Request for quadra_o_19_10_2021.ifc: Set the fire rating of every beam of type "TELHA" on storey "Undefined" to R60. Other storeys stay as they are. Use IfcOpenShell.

First a look at what the model holds.

```python
import ifcopenshell
import ifcopenshell.util.element

model = ifcopenshell.open("quadra_o_19_10_2021.ifc")
print(model.schema)
storey = next(s for s in model.by_type("IfcBuildingStorey") if s.Name == "Undefined")
beams = [e for e in ifcopenshell.util.element.get_decomposition(storey) if e.is_a("IfcBeam")]
seen = {}
for e in beams:
    element_type = ifcopenshell.util.element.get_type(e)
    key = (element_type.Name if element_type != e and element_type else None, ifcopenshell.util.element.get_pset(e, "Pset_BeamCommon", "FireRating"))
    seen[key] = seen.get(key, 0) + 1
for (name, value), count in sorted(seen.items(), key=str):
    print(count, "x", name, "|", value)
```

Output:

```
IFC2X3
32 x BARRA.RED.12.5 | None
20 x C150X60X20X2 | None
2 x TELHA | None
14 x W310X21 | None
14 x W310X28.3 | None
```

```python
import ifcopenshell
import ifcopenshell.api.pset
import ifcopenshell.util.element

model = ifcopenshell.open("quadra_o_19_10_2021.ifc")

storey = next(s for s in model.by_type("IfcBuildingStorey") if s.Name == "Undefined")
beams = [e for e in ifcopenshell.util.element.get_decomposition(storey) if e.is_a("IfcBeam")]

count = 0
for e in beams:
    element_type = ifcopenshell.util.element.get_type(e)
    if element_type in (None, e) or element_type.Name != "TELHA":
        continue
    found = ifcopenshell.util.element.get_pset(e, "Pset_BeamCommon", should_inherit=False)
    if found:
        pset = model.by_id(found["id"])
        if len(ifcopenshell.util.element.get_elements_by_pset(pset)) > 1:
            pset = ifcopenshell.api.pset.unshare_pset(model, products=[e], pset=pset)[0]
    else:
        pset = ifcopenshell.api.pset.add_pset(model, product=e, name="Pset_BeamCommon")
    ifcopenshell.api.pset.edit_pset(model, pset=pset, properties={"FireRating": "R60"})
    count += 1

print(count, "beams updated")

model.write("quadra_o_19_10_2021_updated.ifc")
```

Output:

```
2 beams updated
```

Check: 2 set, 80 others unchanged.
